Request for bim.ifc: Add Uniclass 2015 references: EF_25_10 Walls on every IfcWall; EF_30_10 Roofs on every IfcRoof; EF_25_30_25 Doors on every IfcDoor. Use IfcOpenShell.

First a look at what the model holds.

```python
import ifcopenshell

model = ifcopenshell.open("bim.ifc")
print(model.schema)
print("classifications:", [c.Name for c in model.by_type("IfcClassification")])
for ifc_class in ("IfcDoor", "IfcRoof", "IfcStair", "IfcWall", "IfcWindow"):
    print(ifc_class, len(model.by_type(ifc_class)))
```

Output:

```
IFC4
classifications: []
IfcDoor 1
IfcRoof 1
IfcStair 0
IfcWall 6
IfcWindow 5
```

```python
import ifcopenshell
import ifcopenshell.api.classification

model = ifcopenshell.open("bim.ifc")

system = ifcopenshell.api.classification.add_classification(model, classification="Uniclass 2015")

codes = {
    "IfcWall": ("EF_25_10", "Walls"),
    "IfcRoof": ("EF_30_10", "Roofs"),
    "IfcDoor": ("EF_25_30_25", "Doors"),
}
for ifc_class, (code, name) in codes.items():
    products = model.by_type(ifc_class)
    ifcopenshell.api.classification.add_reference(
        model, products=products, classification=system, identification=code, name=name
    )
    print(code, len(products))

model.write("bim_edited.ifc")
```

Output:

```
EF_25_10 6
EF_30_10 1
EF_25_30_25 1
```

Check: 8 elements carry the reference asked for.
